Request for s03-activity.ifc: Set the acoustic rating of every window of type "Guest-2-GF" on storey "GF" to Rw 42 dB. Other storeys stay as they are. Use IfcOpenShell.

First a look at what the model holds.

```python
import ifcopenshell
import ifcopenshell.util.element

model = ifcopenshell.open("s03-activity.ifc")
print(model.schema)
storey = next(s for s in model.by_type("IfcBuildingStorey") if s.Name == "GF")
windows = [e for e in ifcopenshell.util.element.get_decomposition(storey) if e.is_a("IfcWindow")]
seen = {}
for e in windows:
    element_type = ifcopenshell.util.element.get_type(e)
    key = (element_type.Name if element_type != e and element_type else None, ifcopenshell.util.element.get_pset(e, "Pset_WindowCommon", "AcousticRating"))
    seen[key] = seen.get(key, 0) + 1
for (name, value), count in sorted(seen.items(), key=str):
    print(count, "x", name, "|", value)
```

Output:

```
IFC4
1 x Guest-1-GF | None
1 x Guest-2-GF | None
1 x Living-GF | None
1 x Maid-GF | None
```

```python
import ifcopenshell
import ifcopenshell.api.pset
import ifcopenshell.util.element

model = ifcopenshell.open("s03-activity.ifc")

storey = next(s for s in model.by_type("IfcBuildingStorey") if s.Name == "GF")
windows = [e for e in ifcopenshell.util.element.get_decomposition(storey) if e.is_a("IfcWindow")]

count = 0
for e in windows:
    element_type = ifcopenshell.util.element.get_type(e)
    if element_type in (None, e) or element_type.Name != "Guest-2-GF":
        continue
    # add_pset returns the element's existing set when there is one.
    pset = ifcopenshell.api.pset.add_pset(model, product=e, name="Pset_WindowCommon")
    ifcopenshell.api.pset.edit_pset(model, pset=pset, properties={"AcousticRating": "Rw 42 dB"})
    count += 1

print(count, "windows updated")

model.write("s03-activity_v2.ifc")
```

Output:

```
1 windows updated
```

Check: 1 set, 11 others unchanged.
